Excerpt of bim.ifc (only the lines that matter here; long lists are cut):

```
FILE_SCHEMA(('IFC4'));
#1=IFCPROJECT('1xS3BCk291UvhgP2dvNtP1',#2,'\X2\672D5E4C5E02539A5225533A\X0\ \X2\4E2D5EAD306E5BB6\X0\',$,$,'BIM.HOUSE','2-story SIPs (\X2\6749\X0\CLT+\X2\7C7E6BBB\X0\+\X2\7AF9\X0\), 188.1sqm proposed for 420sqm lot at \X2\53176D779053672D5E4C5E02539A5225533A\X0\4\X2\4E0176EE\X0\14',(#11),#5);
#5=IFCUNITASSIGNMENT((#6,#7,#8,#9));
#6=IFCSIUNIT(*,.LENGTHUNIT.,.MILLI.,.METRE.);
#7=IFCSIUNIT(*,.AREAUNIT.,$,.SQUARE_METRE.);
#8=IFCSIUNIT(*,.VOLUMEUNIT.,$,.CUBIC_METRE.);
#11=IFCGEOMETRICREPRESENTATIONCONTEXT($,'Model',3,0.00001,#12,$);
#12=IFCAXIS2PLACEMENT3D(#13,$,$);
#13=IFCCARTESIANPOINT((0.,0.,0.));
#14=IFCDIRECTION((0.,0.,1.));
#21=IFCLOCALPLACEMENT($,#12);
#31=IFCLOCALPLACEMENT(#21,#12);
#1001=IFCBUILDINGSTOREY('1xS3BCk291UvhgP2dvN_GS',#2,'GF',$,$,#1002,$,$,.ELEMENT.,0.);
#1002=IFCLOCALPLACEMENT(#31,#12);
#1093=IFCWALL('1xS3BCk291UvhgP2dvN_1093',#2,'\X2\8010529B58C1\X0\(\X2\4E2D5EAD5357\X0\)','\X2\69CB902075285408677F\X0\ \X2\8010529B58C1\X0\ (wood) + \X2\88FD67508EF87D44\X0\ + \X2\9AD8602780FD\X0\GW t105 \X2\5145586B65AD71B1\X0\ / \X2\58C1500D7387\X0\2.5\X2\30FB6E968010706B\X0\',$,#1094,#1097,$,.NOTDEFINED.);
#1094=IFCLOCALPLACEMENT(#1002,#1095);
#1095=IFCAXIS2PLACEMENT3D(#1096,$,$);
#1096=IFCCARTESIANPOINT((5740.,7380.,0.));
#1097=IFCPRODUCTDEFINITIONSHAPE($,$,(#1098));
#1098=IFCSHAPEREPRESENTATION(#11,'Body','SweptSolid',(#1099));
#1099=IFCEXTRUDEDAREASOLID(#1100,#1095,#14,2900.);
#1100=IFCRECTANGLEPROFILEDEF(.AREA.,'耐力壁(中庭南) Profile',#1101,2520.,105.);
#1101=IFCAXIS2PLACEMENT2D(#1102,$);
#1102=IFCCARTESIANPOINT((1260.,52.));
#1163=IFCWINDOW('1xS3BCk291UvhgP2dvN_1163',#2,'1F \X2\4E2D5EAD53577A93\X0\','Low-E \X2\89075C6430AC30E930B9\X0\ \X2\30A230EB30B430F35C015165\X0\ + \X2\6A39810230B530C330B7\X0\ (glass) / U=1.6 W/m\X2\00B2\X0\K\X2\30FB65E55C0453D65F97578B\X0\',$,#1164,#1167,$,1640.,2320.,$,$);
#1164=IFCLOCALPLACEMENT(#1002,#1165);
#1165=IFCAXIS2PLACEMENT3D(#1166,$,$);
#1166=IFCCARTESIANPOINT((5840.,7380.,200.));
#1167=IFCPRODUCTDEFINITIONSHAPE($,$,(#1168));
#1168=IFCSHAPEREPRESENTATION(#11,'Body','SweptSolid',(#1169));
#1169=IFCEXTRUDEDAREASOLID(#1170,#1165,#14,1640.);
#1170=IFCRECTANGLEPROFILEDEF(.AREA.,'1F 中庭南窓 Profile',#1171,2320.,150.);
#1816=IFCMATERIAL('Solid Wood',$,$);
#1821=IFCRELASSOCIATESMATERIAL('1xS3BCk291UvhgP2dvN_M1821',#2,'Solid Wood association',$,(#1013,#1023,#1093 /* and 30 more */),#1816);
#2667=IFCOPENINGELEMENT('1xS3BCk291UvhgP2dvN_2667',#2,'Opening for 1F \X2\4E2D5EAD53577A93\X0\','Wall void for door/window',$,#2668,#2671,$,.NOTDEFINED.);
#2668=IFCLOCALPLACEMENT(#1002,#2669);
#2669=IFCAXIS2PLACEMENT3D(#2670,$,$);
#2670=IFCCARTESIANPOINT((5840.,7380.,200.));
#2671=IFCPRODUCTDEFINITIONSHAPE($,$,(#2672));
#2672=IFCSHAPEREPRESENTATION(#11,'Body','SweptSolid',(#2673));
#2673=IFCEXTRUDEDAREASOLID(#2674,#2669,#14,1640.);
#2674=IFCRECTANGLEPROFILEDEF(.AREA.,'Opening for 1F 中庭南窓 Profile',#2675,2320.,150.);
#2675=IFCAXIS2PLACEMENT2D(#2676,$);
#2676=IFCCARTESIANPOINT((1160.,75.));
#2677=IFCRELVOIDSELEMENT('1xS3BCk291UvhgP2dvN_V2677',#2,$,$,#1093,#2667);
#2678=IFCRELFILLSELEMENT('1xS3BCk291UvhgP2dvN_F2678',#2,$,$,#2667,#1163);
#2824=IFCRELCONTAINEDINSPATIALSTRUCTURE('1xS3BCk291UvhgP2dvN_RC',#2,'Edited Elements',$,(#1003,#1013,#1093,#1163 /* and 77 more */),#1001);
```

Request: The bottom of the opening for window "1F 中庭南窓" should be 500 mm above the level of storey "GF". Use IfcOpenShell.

```python
import numpy as np
import ifcopenshell
import ifcopenshell.api.geometry
import ifcopenshell.geom
import ifcopenshell.util.element
import ifcopenshell.util.placement
import ifcopenshell.util.shape
import ifcopenshell.util.unit

model = ifcopenshell.open("bim.ifc")
unit_scale = ifcopenshell.util.unit.calculate_unit_scale(model)

window = model.by_guid("1xS3BCk291UvhgP2dvN_1163")
opening = window.FillsVoids[0].RelatingOpeningElement
storey = ifcopenshell.util.element.get_container(window, ifc_class="IfcBuildingStorey")
level = ifcopenshell.util.placement.get_local_placement(storey.ObjectPlacement)[2, 3]

# The opening's origin need not be at the sill, so measure its lowest point.
shape = ifcopenshell.geom.create_shape(ifcopenshell.geom.settings(), opening)
bottom = ifcopenshell.util.shape.get_shape_bottom_elevation(shape, shape.geometry) / unit_scale
dz = level + 0.5 / unit_scale - bottom

shift = np.array([0.0, 0.0, dz])
# The window is not placed relative to its opening, so move both.
for product in (opening, window):
    matrix = ifcopenshell.util.placement.get_local_placement(product.ObjectPlacement)
    matrix[:3, 3] += shift
    ifcopenshell.api.geometry.edit_object_placement(model, product=product, matrix=matrix, is_si=False)

print(f"moved by {dz * unit_scale:+.3f} m")

model.write("bim_updated.ifc")
```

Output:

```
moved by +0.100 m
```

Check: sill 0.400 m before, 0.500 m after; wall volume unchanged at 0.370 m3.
